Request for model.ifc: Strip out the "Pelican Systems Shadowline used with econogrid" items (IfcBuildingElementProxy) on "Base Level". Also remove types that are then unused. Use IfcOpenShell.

First a look at what the model holds.

```python
import ifcopenshell
import ifcopenshell.util.element

model = ifcopenshell.open("model.ifc")
print(model.schema)
storey = next(s for s in model.by_type("IfcBuildingStorey") if s.Name == "Base Level")
proxies = [e for e in ifcopenshell.util.element.get_decomposition(storey) if e.is_a("IfcBuildingElementProxy")]
seen = {}
for e in proxies:
    element_type = ifcopenshell.util.element.get_type(e)
    name = element_type.Name if element_type not in (None, e) else None
    seen[name] = seen.get(name, 0) + 1
for name, count in sorted(seen.items(), key=str):
    print(count, "x", name)
```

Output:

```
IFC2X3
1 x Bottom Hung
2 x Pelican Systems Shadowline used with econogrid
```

```python
import ifcopenshell
import ifcopenshell.api.root
import ifcopenshell.util.element

model = ifcopenshell.open("model.ifc")

storey = next(s for s in model.by_type("IfcBuildingStorey") if s.Name == "Base Level")
proxies = [e for e in ifcopenshell.util.element.get_decomposition(storey) if e.is_a("IfcBuildingElementProxy")]
targets = [e for e in proxies if (t := ifcopenshell.util.element.get_type(e)) not in (None, e) and t.Name == "Pelican Systems Shadowline used with econogrid"]
types = {ifcopenshell.util.element.get_type(e) for e in targets} - {None, *targets}

for e in targets:
    ifcopenshell.api.root.remove_product(model, product=e)
print(len(targets), "removed")

unused = [t for t in types if not ifcopenshell.util.element.get_types(t)]
for t in unused:
    ifcopenshell.api.root.remove_product(model, product=t)
print(len(unused), "unused types removed")

model.write("model_edited.ifc")
```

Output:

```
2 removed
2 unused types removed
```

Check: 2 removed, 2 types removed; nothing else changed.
